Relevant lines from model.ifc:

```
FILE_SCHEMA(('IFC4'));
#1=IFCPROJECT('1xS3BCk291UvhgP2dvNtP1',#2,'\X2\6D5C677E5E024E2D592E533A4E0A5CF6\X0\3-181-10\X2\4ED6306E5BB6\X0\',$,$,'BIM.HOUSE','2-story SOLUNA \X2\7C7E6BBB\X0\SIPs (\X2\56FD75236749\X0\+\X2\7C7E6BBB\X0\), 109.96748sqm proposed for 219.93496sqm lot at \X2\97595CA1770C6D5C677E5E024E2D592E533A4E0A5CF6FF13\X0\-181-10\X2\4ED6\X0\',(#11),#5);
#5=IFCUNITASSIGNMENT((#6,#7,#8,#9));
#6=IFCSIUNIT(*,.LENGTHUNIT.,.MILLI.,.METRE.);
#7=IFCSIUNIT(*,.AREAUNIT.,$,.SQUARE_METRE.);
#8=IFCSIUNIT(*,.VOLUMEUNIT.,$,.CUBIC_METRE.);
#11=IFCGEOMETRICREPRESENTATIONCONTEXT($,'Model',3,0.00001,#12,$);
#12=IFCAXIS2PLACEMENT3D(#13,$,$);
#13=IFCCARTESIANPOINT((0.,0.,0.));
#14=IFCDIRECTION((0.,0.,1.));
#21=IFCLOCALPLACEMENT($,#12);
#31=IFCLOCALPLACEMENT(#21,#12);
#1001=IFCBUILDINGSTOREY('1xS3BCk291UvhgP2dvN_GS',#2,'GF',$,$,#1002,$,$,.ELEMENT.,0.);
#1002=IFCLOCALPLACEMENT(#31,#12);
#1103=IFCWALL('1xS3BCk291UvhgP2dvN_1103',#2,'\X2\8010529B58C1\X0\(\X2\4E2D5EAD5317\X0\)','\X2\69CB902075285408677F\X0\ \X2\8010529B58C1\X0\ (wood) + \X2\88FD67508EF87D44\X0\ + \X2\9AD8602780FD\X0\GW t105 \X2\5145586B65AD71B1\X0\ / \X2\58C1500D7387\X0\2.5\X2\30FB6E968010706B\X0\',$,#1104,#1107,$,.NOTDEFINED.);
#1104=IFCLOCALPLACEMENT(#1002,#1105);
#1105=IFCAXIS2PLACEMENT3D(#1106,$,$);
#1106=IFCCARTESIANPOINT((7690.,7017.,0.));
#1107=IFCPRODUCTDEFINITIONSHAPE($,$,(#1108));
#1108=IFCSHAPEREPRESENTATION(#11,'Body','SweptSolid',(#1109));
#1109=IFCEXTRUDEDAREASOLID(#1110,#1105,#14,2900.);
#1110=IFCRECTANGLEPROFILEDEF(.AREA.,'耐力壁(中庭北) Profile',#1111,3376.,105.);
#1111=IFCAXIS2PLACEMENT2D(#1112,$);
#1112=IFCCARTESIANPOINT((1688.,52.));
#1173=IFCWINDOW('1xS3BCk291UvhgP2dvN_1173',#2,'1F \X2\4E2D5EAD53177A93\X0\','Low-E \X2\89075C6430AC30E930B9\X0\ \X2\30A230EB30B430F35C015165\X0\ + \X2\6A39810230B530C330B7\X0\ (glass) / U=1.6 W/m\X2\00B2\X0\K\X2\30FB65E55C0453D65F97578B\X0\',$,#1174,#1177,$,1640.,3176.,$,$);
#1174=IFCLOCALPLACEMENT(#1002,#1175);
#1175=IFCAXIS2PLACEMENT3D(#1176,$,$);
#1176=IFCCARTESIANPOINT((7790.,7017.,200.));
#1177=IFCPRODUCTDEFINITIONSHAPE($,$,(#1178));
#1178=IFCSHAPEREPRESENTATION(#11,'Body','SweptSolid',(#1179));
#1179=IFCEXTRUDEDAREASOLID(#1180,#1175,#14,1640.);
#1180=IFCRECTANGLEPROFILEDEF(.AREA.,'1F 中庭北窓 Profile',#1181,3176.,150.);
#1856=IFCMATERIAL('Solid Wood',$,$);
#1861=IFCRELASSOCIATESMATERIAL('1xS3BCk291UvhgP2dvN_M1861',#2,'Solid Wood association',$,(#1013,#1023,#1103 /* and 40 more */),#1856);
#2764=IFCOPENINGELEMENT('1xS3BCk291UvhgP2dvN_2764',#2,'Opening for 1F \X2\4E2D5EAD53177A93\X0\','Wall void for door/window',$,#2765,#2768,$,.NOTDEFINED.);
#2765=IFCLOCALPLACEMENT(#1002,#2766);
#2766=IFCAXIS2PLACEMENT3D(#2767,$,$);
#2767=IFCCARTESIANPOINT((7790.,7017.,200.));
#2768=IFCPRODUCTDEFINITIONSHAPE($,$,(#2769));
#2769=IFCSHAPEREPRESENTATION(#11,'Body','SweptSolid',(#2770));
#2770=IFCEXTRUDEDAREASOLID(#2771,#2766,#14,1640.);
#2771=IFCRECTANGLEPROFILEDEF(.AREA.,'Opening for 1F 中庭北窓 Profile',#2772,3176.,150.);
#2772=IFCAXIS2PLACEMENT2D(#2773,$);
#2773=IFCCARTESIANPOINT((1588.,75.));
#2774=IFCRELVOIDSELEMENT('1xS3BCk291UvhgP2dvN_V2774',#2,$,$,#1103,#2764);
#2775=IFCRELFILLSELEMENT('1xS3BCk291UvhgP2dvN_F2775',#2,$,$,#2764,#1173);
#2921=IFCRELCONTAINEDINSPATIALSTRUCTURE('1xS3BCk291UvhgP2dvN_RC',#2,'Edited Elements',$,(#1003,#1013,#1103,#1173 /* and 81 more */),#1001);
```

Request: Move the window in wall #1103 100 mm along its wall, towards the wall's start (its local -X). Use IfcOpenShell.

```python
import ifcopenshell
import ifcopenshell.api.geometry
import ifcopenshell.util.placement

model = ifcopenshell.open("model.ifc")

window = model.by_guid("1xS3BCk291UvhgP2dvN_1173")
opening = window.FillsVoids[0].RelatingOpeningElement
wall = opening.VoidsElements[0].RelatingBuildingElement

wall_matrix = ifcopenshell.util.placement.get_local_placement(wall.ObjectPlacement)
shift = wall_matrix[:3, 0] * -100.0
before = ifcopenshell.util.placement.get_local_placement(window.ObjectPlacement)[:3, 3].copy()

# The window is not placed relative to its opening, so move both.
for product in (opening, window):
    matrix = ifcopenshell.util.placement.get_local_placement(product.ObjectPlacement)
    matrix[:3, 3] += shift
    ifcopenshell.api.geometry.edit_object_placement(model, product=product, matrix=matrix, is_si=False)

after = ifcopenshell.util.placement.get_local_placement(window.ObjectPlacement)[:3, 3]
print("window moved by", (after - before).round(3) + 0.0)

model.write("model_updated.ifc")
```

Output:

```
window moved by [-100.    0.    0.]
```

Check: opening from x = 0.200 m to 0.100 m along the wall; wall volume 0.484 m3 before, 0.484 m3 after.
